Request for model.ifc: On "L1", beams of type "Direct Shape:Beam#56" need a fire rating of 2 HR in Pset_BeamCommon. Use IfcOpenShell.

First a look at what the model holds.

```python
import ifcopenshell
import ifcopenshell.util.element

model = ifcopenshell.open("model.ifc")
print(model.schema)
storey = next(s for s in model.by_type("IfcBuildingStorey") if s.Name == "L1")
beams = [e for e in ifcopenshell.util.element.get_decomposition(storey) if e.is_a("IfcBeam")]
seen = {}
for e in beams:
    element_type = ifcopenshell.util.element.get_type(e)
    key = (element_type.Name if element_type != e and element_type else None, ifcopenshell.util.element.get_pset(e, "Pset_BeamCommon", "FireRating"))
    seen[key] = seen.get(key, 0) + 1
for (name, value), count in sorted(seen.items(), key=str):
    print(count, "x", name, "|", value)
```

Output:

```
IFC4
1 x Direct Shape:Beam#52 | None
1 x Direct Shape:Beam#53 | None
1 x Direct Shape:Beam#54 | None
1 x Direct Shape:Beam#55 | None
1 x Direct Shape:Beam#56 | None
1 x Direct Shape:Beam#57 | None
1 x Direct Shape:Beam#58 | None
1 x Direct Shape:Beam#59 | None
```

```python
import ifcopenshell
import ifcopenshell.api.pset
import ifcopenshell.util.element

model = ifcopenshell.open("model.ifc")

storey = next(s for s in model.by_type("IfcBuildingStorey") if s.Name == "L1")
beams = [e for e in ifcopenshell.util.element.get_decomposition(storey) if e.is_a("IfcBeam")]

count = 0
for e in beams:
    element_type = ifcopenshell.util.element.get_type(e)
    if element_type in (None, e) or element_type.Name != "Direct Shape:Beam#56":
        continue
    # add_pset returns the element's existing set when there is one.
    pset = ifcopenshell.api.pset.add_pset(model, product=e, name="Pset_BeamCommon")
    ifcopenshell.api.pset.edit_pset(model, pset=pset, properties={"FireRating": "2 HR"})
    count += 1

print(count, "beams updated")

model.write("model_rev.ifc")
```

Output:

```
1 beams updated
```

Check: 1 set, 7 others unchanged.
